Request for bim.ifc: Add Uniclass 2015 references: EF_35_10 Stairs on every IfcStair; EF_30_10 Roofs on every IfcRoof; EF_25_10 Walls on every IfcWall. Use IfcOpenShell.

First a look at what the model holds.

```python
import ifcopenshell

model = ifcopenshell.open("bim.ifc")
print(model.schema)
print("classifications:", [c.Name for c in model.by_type("IfcClassification")])
for ifc_class in ("IfcDoor", "IfcRoof", "IfcStair", "IfcWall", "IfcWindow"):
    print(ifc_class, len(model.by_type(ifc_class)))
```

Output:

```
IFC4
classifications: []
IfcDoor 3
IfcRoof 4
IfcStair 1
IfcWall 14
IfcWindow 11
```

```python
import ifcopenshell
import ifcopenshell.api.classification

model = ifcopenshell.open("bim.ifc")

system = ifcopenshell.api.classification.add_classification(model, classification="Uniclass 2015")

codes = {
    "IfcStair": ("EF_35_10", "Stairs"),
    "IfcRoof": ("EF_30_10", "Roofs"),
    "IfcWall": ("EF_25_10", "Walls"),
}
for ifc_class, (code, name) in codes.items():
    products = model.by_type(ifc_class)
    ifcopenshell.api.classification.add_reference(
        model, products=products, classification=system, identification=code, name=name
    )
    print(code, len(products))

model.write("bim_v2.ifc")
```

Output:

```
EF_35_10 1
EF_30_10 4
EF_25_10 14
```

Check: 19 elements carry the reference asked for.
